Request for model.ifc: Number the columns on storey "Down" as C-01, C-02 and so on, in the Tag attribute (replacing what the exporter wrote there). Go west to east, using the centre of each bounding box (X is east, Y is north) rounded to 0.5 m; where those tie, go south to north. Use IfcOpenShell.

First a look at what the model holds.

```python
import ifcopenshell
import ifcopenshell.util.element
import ifcopenshell.util.placement

model = ifcopenshell.open("model.ifc")
print(model.schema)
storey = next(s for s in model.by_type("IfcBuildingStorey") if s.Name == "Down")
columns = [e for e in ifcopenshell.util.element.get_decomposition(storey) if e.is_a("IfcColumn")]
for e in sorted(columns, key=lambda e: e.id()):
    origin = ifcopenshell.util.placement.get_local_placement(e.ObjectPlacement)[:3, 3]
    print(e.id(), e.Tag, e.Name, origin.round(2) + 0.0, sep=" | ")
```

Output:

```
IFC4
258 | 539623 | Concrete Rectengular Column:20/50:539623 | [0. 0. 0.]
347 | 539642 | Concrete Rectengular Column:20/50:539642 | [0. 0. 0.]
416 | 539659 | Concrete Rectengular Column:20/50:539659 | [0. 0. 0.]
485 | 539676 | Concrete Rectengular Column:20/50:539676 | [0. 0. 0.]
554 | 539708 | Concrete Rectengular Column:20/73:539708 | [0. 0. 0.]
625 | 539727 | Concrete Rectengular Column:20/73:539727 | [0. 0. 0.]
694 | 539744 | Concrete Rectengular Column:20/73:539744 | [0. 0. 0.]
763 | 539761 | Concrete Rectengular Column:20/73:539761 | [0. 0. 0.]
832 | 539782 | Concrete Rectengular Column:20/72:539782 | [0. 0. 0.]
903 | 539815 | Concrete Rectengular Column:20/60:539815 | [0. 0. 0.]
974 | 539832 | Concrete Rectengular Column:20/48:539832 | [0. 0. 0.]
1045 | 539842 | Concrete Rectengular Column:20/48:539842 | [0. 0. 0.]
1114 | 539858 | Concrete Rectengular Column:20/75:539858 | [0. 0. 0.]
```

```python
import ifcopenshell
import ifcopenshell.geom
import ifcopenshell.util.element
import ifcopenshell.util.shape

model = ifcopenshell.open("model.ifc")
settings = ifcopenshell.geom.settings()
settings.set("use-world-coords", True)


def centre(element):
    shape = ifcopenshell.geom.create_shape(settings, element)
    return ifcopenshell.util.shape.get_bbox_centroid(shape.geometry)


storey = next(s for s in model.by_type("IfcBuildingStorey") if s.Name == "Down")
columns = [e for e in ifcopenshell.util.element.get_decomposition(storey) if e.is_a("IfcColumn")]

# Insertion points can sit at a corner or the storey origin, so sort by the geometry (in metres).
centres = {e: centre(e) for e in columns}
columns.sort(key=lambda e: (round(centres[e][0] / 0.5), centres[e][1]))

for i, e in enumerate(columns, start=1):
    number = f"C-{i:02d}"
    e.Tag = number
    print(e.id(), number)

model.write("model_v2.ifc")
```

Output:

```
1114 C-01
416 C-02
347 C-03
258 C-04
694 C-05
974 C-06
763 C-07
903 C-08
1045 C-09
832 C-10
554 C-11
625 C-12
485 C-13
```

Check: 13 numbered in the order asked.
